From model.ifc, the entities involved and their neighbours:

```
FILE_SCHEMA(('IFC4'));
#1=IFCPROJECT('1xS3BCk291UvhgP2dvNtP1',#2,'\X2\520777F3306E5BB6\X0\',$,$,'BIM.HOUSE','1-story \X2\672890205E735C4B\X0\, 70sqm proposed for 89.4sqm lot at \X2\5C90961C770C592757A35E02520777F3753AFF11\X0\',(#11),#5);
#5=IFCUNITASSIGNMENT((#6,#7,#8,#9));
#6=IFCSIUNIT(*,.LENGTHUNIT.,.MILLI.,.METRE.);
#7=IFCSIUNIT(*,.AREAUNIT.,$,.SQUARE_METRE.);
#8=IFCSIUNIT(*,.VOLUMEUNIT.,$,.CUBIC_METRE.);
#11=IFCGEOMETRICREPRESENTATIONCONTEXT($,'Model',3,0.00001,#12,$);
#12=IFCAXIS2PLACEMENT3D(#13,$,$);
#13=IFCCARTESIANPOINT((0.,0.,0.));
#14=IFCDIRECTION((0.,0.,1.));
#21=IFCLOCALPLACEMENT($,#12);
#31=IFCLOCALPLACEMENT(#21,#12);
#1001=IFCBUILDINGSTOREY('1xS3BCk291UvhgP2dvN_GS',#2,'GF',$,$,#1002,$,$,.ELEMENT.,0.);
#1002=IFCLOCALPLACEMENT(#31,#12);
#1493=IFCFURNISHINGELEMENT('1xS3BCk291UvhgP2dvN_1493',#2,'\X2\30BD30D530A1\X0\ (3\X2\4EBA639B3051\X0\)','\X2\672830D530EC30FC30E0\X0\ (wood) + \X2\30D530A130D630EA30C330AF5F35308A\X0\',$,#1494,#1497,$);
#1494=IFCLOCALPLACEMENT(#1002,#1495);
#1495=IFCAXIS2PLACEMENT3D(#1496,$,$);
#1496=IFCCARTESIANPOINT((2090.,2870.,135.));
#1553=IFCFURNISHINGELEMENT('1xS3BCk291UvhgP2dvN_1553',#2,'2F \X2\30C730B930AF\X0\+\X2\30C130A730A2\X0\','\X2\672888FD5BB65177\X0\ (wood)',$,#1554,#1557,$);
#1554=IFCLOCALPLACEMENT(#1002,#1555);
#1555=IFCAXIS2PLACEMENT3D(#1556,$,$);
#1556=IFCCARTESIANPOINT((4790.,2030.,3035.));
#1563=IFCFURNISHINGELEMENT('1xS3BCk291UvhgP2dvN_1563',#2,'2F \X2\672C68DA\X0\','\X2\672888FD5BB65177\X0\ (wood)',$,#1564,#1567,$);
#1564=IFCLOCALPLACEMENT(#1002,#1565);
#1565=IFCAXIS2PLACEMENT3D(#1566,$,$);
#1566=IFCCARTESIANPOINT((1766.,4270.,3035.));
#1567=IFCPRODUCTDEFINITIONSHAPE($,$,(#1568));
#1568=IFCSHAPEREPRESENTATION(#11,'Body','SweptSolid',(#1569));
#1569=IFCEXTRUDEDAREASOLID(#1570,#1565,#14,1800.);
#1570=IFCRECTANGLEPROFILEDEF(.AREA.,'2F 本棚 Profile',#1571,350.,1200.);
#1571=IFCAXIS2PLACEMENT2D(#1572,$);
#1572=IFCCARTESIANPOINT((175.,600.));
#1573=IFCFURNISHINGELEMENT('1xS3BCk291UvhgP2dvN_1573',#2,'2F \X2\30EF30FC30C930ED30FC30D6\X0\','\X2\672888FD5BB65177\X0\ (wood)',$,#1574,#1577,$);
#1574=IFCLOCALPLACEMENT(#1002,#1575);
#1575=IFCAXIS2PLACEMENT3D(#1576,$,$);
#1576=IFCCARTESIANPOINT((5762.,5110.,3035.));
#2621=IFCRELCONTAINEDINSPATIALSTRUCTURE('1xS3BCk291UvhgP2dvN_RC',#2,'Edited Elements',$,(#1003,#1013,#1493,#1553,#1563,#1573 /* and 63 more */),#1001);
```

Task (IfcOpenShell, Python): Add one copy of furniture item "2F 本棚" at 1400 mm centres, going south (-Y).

```python
import numpy as np
import ifcopenshell
import ifcopenshell.api.geometry
import ifcopenshell.api.root
import ifcopenshell.util.element
import ifcopenshell.util.placement

model = ifcopenshell.open("model.ifc")


def reuse_history(source, copy):
    """copy_class also copies each property set's owner history, people and application; keep the originals."""
    for rel in copy.IsDefinedBy:
        if rel.is_a("IfcRelDefinesByProperties") and (history := rel.RelatingPropertyDefinition.OwnerHistory):
            rel.RelatingPropertyDefinition.OwnerHistory = source.OwnerHistory
            ifcopenshell.util.element.remove_deep2(model, history)


source = model.by_id(1563)
base = ifcopenshell.util.placement.get_local_placement(source.ObjectPlacement)
step = np.array([0.0, -1.0, 0.0]) * 1400.0

for i in range(1, 2):
    copy = ifcopenshell.api.root.copy_class(model, product=source)
    copy.Representation = ifcopenshell.util.element.copy_deep(
        model, source.Representation, exclude=["IfcGeometricRepresentationContext", "IfcRepresentationMap"]
    )
    reuse_history(source, copy)
    matrix = base.copy()
    matrix[:3, 3] += i * step
    print("added at", matrix[:3, 3].round(3) + 0.0)
    ifcopenshell.api.geometry.edit_object_placement(model, product=copy, matrix=matrix, is_si=False)

model.write("model_edited.ifc")
```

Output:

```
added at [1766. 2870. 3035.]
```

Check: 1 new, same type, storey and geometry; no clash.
